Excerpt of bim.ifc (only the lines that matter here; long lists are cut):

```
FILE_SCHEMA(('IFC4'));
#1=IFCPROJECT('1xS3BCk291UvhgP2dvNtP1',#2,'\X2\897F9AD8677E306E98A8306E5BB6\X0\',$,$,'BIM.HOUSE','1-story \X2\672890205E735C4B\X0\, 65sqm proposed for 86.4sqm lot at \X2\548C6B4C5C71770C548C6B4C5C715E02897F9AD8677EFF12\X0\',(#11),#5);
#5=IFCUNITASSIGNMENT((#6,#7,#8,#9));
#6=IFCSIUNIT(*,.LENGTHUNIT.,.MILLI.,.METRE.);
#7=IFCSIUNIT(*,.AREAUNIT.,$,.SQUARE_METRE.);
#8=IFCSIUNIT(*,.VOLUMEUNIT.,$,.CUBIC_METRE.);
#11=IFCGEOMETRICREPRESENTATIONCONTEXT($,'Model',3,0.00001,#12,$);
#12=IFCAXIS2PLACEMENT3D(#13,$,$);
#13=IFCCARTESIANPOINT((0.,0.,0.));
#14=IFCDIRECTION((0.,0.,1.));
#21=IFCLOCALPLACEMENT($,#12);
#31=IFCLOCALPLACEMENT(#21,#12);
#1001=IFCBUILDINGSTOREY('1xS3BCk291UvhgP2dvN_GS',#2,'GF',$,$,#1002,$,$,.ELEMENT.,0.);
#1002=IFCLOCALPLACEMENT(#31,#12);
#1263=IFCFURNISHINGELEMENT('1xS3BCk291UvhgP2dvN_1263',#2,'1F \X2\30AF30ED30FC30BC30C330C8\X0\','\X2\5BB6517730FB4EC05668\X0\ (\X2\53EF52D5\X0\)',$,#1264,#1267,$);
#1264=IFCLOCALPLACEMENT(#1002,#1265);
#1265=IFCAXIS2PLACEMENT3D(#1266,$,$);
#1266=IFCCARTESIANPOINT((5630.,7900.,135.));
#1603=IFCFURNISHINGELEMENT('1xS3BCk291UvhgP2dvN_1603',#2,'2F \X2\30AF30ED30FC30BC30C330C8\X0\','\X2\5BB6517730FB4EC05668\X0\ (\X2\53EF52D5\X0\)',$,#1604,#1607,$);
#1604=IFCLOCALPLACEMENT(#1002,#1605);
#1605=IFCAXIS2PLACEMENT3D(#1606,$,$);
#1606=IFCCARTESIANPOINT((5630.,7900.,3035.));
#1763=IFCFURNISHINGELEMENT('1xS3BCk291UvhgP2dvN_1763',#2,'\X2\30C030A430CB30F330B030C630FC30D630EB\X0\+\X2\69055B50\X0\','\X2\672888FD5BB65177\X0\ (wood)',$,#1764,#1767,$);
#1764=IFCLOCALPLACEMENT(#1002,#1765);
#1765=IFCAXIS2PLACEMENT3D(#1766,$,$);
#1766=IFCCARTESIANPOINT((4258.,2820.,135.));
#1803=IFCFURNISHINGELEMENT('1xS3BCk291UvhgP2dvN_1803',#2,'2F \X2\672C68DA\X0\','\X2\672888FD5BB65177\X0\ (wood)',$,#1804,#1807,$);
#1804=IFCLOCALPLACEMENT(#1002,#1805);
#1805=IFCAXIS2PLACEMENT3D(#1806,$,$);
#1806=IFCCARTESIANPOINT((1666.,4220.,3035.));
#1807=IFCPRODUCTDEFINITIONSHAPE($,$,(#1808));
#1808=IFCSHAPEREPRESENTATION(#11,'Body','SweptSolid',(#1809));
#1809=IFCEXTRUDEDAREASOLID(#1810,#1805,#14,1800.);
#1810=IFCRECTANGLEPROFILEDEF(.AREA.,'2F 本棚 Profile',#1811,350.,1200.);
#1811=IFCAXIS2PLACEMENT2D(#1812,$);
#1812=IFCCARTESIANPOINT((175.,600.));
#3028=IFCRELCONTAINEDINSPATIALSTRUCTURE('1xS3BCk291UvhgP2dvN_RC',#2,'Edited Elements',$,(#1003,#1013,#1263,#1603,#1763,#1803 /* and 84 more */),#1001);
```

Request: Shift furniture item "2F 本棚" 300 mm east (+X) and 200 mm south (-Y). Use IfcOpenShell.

```python
import ifcopenshell
import ifcopenshell.api.geometry
import ifcopenshell.util.placement
import ifcopenshell.util.unit

model = ifcopenshell.open("bim.ifc")
unit_scale = ifcopenshell.util.unit.calculate_unit_scale(model)

item = model.by_id(1803)
matrix = ifcopenshell.util.placement.get_local_placement(item.ObjectPlacement)
matrix[0, 3] += 0.3 / unit_scale
matrix[1, 3] -= 0.2 / unit_scale
ifcopenshell.api.geometry.edit_object_placement(model, product=item, matrix=matrix, is_si=False)

print(ifcopenshell.util.placement.get_local_placement(item.ObjectPlacement).round(3) + 0.0)

model.write("bim-out.ifc")
```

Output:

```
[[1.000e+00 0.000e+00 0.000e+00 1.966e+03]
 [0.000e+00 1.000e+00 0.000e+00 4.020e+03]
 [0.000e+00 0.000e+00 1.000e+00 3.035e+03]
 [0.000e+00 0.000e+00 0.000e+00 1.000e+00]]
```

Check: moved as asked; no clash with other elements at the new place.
